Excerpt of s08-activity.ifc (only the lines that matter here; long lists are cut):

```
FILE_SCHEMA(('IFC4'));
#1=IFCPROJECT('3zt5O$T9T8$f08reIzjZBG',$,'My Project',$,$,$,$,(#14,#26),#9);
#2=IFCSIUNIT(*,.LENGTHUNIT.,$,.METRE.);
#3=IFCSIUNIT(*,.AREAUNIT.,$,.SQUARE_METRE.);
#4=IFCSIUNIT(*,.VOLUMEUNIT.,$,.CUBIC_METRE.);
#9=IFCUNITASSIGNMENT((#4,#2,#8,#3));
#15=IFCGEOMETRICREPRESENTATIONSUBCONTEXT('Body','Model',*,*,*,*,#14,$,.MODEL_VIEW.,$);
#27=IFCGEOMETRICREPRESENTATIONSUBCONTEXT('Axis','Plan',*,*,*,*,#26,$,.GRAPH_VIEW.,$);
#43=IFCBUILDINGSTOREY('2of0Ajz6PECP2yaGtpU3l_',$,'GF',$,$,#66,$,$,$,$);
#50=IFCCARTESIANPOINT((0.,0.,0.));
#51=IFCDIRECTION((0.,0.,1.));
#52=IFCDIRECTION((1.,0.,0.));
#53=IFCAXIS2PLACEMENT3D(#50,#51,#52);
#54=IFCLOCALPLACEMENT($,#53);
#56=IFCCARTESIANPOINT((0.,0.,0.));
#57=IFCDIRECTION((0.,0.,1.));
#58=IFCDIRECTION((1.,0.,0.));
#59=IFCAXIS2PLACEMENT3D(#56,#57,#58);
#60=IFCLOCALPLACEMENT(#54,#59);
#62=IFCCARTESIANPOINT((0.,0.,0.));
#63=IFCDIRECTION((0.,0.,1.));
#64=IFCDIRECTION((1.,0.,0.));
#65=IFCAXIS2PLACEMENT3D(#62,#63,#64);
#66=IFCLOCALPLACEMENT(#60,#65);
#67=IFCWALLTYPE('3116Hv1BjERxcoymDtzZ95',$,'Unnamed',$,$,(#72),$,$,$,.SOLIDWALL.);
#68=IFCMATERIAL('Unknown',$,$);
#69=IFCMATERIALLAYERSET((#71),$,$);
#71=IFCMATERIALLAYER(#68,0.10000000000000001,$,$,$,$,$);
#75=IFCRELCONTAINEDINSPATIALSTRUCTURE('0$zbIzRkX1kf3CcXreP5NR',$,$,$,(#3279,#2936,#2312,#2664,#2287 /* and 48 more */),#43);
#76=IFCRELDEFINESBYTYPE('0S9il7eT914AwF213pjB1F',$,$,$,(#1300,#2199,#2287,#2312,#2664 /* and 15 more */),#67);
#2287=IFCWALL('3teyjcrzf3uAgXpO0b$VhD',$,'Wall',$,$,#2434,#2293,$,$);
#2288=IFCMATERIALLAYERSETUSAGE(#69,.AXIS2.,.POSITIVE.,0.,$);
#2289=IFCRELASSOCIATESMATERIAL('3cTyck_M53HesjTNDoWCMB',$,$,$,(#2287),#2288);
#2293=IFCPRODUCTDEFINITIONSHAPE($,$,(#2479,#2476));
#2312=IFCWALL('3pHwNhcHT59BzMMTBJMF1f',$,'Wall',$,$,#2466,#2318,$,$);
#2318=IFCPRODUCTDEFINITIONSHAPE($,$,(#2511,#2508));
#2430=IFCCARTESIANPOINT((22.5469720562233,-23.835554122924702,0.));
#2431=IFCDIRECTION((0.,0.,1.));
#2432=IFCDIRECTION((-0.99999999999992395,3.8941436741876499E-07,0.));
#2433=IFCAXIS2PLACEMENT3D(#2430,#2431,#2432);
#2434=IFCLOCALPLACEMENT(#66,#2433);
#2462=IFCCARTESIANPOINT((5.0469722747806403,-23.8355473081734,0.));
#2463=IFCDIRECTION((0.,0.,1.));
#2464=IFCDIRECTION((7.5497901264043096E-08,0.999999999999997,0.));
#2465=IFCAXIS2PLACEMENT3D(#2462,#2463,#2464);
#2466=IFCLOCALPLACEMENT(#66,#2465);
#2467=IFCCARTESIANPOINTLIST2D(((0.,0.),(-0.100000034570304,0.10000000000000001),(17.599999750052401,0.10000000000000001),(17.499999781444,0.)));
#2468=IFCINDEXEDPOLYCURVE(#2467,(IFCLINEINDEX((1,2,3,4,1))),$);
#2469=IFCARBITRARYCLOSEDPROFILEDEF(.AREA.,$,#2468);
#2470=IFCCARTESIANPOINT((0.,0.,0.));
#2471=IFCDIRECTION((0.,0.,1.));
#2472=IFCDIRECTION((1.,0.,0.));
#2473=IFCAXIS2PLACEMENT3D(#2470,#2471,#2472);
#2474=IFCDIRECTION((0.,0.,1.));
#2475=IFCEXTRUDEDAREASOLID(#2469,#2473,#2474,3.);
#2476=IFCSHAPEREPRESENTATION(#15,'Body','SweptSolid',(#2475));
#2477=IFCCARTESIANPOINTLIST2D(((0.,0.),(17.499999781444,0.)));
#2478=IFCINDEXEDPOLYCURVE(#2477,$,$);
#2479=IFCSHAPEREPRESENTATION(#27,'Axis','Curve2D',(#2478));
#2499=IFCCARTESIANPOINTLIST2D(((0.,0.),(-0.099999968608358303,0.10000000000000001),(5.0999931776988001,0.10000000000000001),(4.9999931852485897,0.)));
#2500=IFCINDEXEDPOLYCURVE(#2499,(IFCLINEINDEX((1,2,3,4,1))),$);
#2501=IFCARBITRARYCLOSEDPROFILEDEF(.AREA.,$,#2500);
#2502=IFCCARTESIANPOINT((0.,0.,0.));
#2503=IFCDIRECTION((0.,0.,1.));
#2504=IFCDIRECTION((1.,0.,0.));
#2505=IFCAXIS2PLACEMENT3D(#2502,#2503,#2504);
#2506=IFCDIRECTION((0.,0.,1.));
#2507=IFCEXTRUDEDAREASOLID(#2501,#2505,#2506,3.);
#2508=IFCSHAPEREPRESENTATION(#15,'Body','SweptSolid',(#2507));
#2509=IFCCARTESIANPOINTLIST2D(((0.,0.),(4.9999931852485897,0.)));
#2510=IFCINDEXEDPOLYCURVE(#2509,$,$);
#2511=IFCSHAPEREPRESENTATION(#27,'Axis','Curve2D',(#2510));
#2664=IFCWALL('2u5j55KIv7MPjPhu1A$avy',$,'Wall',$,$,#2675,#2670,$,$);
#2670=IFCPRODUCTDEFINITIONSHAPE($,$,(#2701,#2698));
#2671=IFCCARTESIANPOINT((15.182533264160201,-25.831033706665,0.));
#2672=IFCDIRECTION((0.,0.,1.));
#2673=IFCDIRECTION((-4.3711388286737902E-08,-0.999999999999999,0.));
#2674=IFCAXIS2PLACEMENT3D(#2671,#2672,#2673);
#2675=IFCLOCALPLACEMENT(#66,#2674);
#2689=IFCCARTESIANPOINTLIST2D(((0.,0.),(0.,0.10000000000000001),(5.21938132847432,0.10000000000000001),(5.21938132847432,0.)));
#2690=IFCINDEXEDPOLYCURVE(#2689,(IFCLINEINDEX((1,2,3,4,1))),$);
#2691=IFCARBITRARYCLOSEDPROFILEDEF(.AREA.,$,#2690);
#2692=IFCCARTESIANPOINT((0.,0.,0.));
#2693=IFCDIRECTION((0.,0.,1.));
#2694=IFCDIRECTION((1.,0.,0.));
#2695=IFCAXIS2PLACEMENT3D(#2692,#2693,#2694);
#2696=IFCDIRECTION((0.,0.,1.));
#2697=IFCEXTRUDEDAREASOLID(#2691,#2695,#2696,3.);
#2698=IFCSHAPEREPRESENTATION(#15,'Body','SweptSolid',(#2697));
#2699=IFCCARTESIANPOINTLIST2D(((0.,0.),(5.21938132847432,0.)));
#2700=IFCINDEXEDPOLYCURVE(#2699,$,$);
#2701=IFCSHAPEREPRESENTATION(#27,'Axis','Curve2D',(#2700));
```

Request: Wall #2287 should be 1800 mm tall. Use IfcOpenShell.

```python
import ifcopenshell
import ifcopenshell.geom
import ifcopenshell.util.representation
import ifcopenshell.util.shape
import ifcopenshell.util.unit

model = ifcopenshell.open("s08-activity.ifc")
unit_scale = ifcopenshell.util.unit.calculate_unit_scale(model)
settings = ifcopenshell.geom.settings()


def volume(element):
    """Net volume in cubic metres, openings subtracted."""
    shape = ifcopenshell.geom.create_shape(settings, element)
    return ifcopenshell.util.shape.get_volume(shape.geometry)


wall = model.by_guid("3teyjcrzf3uAgXpO0b$VhD")
before = volume(wall)

body = ifcopenshell.util.representation.get_representation(wall, "Model", "Body")
solid = body.Items[0]
old_height = solid.Depth
solid.Depth = 1.8 / unit_scale
after = volume(wall)

print(f"height {old_height:g} -> {solid.Depth:g}, volume {before:.3f} -> {after:.3f} m3")

model.write("s08-activity_updated.ifc")
```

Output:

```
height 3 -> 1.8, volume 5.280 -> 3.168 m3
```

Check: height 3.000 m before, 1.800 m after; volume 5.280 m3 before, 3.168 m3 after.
